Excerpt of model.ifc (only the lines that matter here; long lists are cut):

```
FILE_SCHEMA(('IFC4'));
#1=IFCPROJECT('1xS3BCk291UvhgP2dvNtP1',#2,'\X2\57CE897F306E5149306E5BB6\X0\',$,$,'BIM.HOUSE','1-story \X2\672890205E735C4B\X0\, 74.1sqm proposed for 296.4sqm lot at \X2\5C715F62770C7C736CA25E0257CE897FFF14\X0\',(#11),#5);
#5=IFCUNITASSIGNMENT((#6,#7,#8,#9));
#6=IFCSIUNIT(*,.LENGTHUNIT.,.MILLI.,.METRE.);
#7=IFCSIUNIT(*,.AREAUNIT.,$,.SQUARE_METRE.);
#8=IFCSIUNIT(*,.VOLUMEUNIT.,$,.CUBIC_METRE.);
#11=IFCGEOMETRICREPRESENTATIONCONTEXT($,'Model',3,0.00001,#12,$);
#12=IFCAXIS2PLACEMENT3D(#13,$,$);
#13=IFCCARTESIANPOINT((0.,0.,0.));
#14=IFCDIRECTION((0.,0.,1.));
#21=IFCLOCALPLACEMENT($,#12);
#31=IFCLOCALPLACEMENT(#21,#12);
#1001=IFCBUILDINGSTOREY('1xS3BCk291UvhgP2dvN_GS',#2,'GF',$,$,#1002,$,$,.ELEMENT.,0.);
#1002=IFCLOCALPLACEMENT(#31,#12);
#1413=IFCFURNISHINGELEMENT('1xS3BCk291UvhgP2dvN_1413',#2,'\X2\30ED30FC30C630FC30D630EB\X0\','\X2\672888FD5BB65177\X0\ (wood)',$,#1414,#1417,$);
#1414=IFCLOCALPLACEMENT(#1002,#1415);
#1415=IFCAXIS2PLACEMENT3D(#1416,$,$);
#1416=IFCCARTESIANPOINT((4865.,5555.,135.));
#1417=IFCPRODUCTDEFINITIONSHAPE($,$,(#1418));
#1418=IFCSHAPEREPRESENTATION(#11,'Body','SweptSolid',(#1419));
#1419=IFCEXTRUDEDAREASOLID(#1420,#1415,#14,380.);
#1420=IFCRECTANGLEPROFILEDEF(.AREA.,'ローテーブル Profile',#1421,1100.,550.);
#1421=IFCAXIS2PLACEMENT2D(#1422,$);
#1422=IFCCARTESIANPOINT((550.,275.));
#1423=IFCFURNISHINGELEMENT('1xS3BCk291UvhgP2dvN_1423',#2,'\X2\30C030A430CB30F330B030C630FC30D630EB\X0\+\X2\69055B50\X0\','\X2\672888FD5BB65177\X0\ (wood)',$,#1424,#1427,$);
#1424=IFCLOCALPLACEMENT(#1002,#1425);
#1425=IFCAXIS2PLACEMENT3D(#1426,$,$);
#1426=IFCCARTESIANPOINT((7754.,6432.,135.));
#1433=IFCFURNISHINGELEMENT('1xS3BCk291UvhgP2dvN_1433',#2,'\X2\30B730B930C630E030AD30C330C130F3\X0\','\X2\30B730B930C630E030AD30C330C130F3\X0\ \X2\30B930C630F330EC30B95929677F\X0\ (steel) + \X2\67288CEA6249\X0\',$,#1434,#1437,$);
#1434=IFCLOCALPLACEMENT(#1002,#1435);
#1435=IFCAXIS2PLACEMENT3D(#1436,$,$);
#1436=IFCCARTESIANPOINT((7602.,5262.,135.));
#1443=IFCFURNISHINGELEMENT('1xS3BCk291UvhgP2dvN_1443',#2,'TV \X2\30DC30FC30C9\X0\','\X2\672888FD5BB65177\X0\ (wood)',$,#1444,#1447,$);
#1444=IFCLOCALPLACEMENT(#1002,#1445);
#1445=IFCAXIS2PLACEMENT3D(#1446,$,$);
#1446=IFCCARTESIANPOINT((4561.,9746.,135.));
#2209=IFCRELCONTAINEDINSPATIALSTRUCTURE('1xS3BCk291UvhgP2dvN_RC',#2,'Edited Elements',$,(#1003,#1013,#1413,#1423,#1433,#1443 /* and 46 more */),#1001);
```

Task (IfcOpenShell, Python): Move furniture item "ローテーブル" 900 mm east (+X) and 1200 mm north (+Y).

```python
import ifcopenshell
import ifcopenshell.api.geometry
import ifcopenshell.util.placement
import ifcopenshell.util.unit

model = ifcopenshell.open("model.ifc")
unit_scale = ifcopenshell.util.unit.calculate_unit_scale(model)

item = model.by_guid("1xS3BCk291UvhgP2dvN_1413")
matrix = ifcopenshell.util.placement.get_local_placement(item.ObjectPlacement)
matrix[0, 3] += 0.9 / unit_scale
matrix[1, 3] += 1.2 / unit_scale
ifcopenshell.api.geometry.edit_object_placement(model, product=item, matrix=matrix, is_si=False)

print(ifcopenshell.util.placement.get_local_placement(item.ObjectPlacement).round(3) + 0.0)

model.write("model_edited.ifc")
```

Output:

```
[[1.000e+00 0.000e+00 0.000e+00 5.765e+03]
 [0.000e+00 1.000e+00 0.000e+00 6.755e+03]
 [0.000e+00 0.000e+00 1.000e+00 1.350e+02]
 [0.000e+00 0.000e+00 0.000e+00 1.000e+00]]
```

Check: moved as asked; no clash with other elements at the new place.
